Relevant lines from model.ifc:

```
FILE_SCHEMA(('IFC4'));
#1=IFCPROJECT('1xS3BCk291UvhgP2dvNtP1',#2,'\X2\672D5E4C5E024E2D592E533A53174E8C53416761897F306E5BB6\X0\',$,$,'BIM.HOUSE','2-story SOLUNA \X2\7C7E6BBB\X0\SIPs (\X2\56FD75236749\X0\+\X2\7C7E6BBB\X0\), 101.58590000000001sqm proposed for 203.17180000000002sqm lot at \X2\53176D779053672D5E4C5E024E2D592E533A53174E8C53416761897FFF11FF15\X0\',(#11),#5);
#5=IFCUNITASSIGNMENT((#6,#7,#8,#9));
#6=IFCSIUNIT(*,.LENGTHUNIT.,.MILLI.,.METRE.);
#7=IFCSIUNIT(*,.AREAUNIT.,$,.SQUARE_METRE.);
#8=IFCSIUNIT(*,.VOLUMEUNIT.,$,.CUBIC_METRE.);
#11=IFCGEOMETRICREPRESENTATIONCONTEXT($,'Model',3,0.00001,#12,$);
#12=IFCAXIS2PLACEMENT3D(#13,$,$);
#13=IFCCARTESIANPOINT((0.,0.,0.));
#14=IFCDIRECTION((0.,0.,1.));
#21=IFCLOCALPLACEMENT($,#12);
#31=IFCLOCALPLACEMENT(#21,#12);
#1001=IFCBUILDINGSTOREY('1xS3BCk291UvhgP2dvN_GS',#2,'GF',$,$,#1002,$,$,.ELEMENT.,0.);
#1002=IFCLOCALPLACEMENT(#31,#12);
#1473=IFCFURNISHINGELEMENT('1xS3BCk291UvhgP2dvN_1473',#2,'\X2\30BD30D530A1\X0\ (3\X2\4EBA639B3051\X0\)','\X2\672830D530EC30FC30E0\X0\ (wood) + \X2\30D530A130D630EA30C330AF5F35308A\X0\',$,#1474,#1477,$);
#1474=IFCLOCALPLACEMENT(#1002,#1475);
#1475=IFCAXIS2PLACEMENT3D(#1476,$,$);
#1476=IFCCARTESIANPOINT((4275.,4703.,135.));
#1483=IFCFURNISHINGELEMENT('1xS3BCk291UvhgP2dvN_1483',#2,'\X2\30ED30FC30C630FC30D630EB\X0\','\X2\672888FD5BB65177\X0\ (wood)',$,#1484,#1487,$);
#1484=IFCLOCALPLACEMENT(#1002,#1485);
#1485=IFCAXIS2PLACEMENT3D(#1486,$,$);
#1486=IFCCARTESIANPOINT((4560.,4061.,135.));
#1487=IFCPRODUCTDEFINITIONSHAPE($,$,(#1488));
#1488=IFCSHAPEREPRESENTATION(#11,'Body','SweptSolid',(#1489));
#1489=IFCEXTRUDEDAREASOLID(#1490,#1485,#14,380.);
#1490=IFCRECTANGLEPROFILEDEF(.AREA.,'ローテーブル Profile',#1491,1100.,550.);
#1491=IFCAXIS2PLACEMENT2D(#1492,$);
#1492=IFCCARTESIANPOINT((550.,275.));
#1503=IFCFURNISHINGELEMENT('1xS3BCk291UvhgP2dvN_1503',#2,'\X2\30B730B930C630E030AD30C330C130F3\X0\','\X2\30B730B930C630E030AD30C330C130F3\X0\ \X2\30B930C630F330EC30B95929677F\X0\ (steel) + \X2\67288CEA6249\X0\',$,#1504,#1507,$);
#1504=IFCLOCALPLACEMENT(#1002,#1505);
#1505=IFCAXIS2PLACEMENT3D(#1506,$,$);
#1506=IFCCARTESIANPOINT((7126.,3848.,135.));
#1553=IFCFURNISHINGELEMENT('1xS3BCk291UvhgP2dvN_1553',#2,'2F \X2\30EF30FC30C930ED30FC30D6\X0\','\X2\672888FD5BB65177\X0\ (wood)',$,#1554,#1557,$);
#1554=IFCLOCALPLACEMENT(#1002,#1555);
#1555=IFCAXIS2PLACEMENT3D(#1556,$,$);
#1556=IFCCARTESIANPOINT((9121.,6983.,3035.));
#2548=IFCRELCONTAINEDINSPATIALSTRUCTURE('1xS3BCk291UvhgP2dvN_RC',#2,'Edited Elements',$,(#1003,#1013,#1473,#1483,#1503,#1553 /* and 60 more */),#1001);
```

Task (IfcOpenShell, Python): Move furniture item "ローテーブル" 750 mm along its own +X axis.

```python
import ifcopenshell
import ifcopenshell.api.geometry
import ifcopenshell.util.placement
import ifcopenshell.util.unit

model = ifcopenshell.open("model.ifc")
unit_scale = ifcopenshell.util.unit.calculate_unit_scale(model)

item = model.by_guid("1xS3BCk291UvhgP2dvN_1483")
matrix = ifcopenshell.util.placement.get_local_placement(item.ObjectPlacement)
matrix[:3, 3] += matrix[:3, 0] * 0.75 / unit_scale
ifcopenshell.api.geometry.edit_object_placement(model, product=item, matrix=matrix, is_si=False)

print(ifcopenshell.util.placement.get_local_placement(item.ObjectPlacement).round(3) + 0.0)

model.write("model_updated.ifc")
```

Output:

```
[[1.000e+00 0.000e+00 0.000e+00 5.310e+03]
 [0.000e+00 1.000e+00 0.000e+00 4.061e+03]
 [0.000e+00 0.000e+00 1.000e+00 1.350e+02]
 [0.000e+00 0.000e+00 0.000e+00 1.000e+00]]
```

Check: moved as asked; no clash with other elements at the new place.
